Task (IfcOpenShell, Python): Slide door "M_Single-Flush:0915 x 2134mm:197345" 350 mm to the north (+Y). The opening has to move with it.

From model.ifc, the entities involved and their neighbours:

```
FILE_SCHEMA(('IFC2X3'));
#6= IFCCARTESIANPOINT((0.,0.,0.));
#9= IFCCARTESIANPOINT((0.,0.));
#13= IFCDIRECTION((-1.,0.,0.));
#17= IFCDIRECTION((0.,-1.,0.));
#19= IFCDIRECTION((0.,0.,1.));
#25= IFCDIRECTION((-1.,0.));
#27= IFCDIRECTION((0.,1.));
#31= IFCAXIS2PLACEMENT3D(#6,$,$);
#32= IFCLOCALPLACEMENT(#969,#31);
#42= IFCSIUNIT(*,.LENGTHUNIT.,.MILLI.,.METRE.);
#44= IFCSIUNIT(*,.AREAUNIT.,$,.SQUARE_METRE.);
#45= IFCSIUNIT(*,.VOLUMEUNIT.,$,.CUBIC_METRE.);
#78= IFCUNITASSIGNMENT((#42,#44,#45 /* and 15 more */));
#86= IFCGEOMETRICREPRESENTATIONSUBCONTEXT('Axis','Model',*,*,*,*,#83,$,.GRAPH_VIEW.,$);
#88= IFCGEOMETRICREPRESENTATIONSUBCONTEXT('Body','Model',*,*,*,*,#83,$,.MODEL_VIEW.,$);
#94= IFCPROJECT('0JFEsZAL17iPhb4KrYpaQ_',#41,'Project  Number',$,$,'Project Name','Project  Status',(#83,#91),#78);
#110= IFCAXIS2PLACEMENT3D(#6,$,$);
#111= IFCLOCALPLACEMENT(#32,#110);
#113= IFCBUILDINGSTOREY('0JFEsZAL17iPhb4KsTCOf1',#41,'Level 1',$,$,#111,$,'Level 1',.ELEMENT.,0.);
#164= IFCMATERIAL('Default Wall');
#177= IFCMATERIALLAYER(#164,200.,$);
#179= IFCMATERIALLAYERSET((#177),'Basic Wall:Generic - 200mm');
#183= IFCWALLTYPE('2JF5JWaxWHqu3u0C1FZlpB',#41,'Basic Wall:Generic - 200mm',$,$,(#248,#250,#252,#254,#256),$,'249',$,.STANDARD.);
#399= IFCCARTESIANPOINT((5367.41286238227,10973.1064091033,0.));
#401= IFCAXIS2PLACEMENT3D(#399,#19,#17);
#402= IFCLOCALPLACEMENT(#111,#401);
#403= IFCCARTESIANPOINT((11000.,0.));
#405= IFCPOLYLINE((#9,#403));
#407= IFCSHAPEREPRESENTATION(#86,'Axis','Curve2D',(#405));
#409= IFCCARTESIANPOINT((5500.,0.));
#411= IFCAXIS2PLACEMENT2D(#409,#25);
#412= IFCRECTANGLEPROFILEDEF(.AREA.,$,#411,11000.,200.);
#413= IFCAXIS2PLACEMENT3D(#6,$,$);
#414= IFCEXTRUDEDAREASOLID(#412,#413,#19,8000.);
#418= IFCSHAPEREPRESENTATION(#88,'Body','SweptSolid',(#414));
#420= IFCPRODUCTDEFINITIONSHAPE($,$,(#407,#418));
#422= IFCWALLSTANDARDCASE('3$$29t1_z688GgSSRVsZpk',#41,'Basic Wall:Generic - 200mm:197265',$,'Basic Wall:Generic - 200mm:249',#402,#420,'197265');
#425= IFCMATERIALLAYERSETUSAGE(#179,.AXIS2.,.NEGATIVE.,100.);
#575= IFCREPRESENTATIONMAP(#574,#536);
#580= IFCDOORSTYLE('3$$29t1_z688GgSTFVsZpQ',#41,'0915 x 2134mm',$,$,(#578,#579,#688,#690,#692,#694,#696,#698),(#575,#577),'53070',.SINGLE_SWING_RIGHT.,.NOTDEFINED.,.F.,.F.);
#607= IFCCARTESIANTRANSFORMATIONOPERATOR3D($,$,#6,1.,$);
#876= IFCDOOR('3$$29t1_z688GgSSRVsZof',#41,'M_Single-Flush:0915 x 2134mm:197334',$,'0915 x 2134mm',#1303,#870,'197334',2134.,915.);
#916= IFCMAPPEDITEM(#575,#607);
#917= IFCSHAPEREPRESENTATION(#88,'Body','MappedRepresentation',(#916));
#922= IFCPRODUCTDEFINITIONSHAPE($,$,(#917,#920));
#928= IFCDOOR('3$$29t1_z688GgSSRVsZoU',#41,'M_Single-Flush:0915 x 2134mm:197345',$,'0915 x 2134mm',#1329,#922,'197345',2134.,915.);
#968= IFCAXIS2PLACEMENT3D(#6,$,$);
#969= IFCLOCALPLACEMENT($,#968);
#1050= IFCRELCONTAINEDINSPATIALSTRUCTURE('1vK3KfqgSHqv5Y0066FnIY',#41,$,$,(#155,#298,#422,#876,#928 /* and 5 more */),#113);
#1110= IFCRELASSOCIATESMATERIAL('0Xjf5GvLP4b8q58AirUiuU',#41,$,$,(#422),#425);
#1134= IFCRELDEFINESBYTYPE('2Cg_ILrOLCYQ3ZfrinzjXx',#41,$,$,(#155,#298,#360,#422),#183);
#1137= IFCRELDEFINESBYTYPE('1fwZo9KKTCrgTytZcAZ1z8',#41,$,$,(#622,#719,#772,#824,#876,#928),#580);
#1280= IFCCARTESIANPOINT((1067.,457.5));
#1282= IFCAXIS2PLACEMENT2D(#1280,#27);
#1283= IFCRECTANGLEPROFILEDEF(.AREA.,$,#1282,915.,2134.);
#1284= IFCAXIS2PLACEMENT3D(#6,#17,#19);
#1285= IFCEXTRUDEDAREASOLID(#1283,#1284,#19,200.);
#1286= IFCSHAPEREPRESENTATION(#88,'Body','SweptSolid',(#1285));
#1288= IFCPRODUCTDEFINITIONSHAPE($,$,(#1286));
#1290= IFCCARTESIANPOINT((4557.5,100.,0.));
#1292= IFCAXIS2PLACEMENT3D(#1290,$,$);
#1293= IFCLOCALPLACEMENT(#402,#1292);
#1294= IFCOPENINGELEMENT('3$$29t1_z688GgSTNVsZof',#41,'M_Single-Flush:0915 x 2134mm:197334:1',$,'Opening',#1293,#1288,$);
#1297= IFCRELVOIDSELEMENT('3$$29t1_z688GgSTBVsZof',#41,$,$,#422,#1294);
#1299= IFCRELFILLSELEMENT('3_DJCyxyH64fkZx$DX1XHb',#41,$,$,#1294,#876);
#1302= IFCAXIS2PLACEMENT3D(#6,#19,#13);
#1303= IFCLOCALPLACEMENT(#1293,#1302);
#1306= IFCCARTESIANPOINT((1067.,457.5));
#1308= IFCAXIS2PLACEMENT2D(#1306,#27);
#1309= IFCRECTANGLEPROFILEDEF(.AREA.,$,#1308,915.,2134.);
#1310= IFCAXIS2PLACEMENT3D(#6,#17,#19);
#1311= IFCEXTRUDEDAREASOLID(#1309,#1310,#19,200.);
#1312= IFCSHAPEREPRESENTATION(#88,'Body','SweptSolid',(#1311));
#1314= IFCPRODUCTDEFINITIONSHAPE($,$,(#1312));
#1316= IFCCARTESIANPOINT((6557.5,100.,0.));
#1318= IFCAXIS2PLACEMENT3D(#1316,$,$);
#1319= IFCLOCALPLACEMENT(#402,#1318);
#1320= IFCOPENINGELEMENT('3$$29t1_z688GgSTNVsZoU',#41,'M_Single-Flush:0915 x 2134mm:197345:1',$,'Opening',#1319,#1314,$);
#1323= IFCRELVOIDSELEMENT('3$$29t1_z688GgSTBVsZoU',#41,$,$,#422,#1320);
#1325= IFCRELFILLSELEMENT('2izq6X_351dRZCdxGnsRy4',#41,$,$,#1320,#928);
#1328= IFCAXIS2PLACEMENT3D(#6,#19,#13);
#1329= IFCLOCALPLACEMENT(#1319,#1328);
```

```python
import ifcopenshell
import ifcopenshell.api.geometry
import ifcopenshell.util.placement
import ifcopenshell.util.unit

model = ifcopenshell.open("model.ifc")
unit_scale = ifcopenshell.util.unit.calculate_unit_scale(model)

door = model.by_guid("3$$29t1_z688GgSSRVsZoU")
opening = door.FillsVoids[0].RelatingOpeningElement
wall = opening.VoidsElements[0].RelatingBuildingElement

wall_matrix = ifcopenshell.util.placement.get_local_placement(wall.ObjectPlacement)
shift = wall_matrix[:3, 0] * -0.35 / unit_scale
before = ifcopenshell.util.placement.get_local_placement(door.ObjectPlacement)[:3, 3].copy()

# The door is placed relative to its opening, so it follows when the opening moves.
matrix = ifcopenshell.util.placement.get_local_placement(opening.ObjectPlacement)
matrix[:3, 3] += shift
ifcopenshell.api.geometry.edit_object_placement(
    model, product=opening, matrix=matrix, is_si=False, should_transform_children=True
)

after = ifcopenshell.util.placement.get_local_placement(door.ObjectPlacement)[:3, 3]
print("door moved by", (after - before).round(3) + 0.0)

model.write("model_updated.ifc")
```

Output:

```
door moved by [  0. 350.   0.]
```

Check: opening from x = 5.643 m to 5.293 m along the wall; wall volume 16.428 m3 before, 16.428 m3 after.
